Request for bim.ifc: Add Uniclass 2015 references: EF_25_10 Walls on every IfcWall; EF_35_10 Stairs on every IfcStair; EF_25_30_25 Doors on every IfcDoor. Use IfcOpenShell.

First a look at what the model holds.

```python
import ifcopenshell

model = ifcopenshell.open("bim.ifc")
print(model.schema)
print("classifications:", [c.Name for c in model.by_type("IfcClassification")])
for ifc_class in ("IfcDoor", "IfcRoof", "IfcStair", "IfcWall", "IfcWindow"):
    print(ifc_class, len(model.by_type(ifc_class)))
```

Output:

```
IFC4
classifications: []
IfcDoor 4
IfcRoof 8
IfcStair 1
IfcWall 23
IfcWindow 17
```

```python
import ifcopenshell
import ifcopenshell.api.classification

model = ifcopenshell.open("bim.ifc")

system = ifcopenshell.api.classification.add_classification(model, classification="Uniclass 2015")

codes = {
    "IfcWall": ("EF_25_10", "Walls"),
    "IfcStair": ("EF_35_10", "Stairs"),
    "IfcDoor": ("EF_25_30_25", "Doors"),
}
for ifc_class, (code, name) in codes.items():
    products = model.by_type(ifc_class)
    ifcopenshell.api.classification.add_reference(
        model, products=products, classification=system, identification=code, name=name
    )
    print(code, len(products))

model.write("bim-out.ifc")
```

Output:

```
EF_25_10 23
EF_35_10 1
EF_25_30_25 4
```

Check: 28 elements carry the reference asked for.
